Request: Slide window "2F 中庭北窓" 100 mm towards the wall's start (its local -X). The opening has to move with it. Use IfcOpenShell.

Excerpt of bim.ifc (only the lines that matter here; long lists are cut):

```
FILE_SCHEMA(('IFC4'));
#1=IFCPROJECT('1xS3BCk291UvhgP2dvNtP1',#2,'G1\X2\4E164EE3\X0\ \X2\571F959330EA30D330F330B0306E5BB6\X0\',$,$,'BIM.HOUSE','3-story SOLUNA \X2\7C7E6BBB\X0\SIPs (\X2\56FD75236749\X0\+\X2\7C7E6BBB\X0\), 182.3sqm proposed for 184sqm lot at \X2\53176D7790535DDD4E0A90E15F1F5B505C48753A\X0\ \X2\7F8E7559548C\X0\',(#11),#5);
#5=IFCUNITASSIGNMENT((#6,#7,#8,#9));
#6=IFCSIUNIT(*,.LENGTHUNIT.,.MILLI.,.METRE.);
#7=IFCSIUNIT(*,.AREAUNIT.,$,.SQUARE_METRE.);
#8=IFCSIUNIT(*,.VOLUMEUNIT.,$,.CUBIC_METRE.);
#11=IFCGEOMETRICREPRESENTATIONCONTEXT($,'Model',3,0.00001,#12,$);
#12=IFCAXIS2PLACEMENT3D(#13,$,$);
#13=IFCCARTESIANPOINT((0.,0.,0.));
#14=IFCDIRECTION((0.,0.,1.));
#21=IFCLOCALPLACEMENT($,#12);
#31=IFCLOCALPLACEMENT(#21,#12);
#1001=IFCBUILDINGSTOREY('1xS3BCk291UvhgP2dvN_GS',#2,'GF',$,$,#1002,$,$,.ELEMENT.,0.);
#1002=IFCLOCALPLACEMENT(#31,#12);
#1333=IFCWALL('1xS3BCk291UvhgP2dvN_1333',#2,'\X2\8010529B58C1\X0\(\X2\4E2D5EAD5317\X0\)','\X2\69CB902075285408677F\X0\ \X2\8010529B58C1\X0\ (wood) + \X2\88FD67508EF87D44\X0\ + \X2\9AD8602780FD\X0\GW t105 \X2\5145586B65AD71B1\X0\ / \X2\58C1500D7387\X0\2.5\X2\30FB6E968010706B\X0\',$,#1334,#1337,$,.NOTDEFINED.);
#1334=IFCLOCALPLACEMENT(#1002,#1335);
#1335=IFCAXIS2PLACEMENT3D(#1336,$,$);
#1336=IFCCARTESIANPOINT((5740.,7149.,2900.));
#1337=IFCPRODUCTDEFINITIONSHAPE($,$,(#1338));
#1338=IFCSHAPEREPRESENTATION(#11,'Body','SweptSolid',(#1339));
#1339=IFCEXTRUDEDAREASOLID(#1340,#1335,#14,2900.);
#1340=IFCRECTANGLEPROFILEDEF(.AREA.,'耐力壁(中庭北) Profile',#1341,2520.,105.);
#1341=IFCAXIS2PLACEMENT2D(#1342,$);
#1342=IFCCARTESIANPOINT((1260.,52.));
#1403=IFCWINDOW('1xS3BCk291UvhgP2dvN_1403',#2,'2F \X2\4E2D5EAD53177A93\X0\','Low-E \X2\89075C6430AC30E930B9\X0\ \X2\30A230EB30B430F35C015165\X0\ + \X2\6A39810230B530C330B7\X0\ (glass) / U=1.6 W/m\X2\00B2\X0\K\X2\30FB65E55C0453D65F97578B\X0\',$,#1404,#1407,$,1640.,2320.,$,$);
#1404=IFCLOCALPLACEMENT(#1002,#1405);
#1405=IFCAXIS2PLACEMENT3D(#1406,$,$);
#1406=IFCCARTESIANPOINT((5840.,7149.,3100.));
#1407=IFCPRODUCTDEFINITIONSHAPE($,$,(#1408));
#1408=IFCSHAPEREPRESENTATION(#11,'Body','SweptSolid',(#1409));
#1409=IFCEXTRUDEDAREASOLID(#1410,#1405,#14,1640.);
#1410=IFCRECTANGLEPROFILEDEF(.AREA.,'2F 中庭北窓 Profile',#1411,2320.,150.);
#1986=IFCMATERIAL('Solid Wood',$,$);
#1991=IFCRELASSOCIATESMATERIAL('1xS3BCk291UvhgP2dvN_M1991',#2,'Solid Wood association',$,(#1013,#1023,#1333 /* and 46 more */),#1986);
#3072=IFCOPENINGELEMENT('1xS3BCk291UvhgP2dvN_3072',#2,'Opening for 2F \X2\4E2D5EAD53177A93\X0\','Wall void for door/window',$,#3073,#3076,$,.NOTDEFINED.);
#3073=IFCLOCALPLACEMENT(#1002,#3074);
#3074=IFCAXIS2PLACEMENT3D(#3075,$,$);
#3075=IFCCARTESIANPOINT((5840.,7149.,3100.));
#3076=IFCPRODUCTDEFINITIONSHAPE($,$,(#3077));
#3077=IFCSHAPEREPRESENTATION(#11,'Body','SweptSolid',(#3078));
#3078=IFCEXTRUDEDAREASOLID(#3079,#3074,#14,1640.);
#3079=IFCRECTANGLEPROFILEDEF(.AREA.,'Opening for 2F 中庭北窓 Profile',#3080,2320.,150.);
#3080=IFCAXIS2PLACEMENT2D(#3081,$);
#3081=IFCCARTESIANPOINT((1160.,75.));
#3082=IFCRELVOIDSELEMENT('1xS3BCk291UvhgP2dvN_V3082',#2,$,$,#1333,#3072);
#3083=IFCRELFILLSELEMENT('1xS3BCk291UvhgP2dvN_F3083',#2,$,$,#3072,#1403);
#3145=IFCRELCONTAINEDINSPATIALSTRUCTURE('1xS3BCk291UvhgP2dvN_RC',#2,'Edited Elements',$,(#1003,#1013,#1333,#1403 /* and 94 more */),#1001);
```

```python
import ifcopenshell
import ifcopenshell.api.geometry
import ifcopenshell.util.placement
import ifcopenshell.util.unit

model = ifcopenshell.open("bim.ifc")
unit_scale = ifcopenshell.util.unit.calculate_unit_scale(model)

window = model.by_id(1403)
opening = window.FillsVoids[0].RelatingOpeningElement
wall = opening.VoidsElements[0].RelatingBuildingElement

wall_matrix = ifcopenshell.util.placement.get_local_placement(wall.ObjectPlacement)
shift = wall_matrix[:3, 0] * -0.1 / unit_scale
before = ifcopenshell.util.placement.get_local_placement(window.ObjectPlacement)[:3, 3].copy()

# The window is not placed relative to its opening, so move both.
for product in (opening, window):
    matrix = ifcopenshell.util.placement.get_local_placement(product.ObjectPlacement)
    matrix[:3, 3] += shift
    ifcopenshell.api.geometry.edit_object_placement(model, product=product, matrix=matrix, is_si=False)

after = ifcopenshell.util.placement.get_local_placement(window.ObjectPlacement)[:3, 3]
print("window moved by", (after - before).round(3) + 0.0)

model.write("bim_rev.ifc")
```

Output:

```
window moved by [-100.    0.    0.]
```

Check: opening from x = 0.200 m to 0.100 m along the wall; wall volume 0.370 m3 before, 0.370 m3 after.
